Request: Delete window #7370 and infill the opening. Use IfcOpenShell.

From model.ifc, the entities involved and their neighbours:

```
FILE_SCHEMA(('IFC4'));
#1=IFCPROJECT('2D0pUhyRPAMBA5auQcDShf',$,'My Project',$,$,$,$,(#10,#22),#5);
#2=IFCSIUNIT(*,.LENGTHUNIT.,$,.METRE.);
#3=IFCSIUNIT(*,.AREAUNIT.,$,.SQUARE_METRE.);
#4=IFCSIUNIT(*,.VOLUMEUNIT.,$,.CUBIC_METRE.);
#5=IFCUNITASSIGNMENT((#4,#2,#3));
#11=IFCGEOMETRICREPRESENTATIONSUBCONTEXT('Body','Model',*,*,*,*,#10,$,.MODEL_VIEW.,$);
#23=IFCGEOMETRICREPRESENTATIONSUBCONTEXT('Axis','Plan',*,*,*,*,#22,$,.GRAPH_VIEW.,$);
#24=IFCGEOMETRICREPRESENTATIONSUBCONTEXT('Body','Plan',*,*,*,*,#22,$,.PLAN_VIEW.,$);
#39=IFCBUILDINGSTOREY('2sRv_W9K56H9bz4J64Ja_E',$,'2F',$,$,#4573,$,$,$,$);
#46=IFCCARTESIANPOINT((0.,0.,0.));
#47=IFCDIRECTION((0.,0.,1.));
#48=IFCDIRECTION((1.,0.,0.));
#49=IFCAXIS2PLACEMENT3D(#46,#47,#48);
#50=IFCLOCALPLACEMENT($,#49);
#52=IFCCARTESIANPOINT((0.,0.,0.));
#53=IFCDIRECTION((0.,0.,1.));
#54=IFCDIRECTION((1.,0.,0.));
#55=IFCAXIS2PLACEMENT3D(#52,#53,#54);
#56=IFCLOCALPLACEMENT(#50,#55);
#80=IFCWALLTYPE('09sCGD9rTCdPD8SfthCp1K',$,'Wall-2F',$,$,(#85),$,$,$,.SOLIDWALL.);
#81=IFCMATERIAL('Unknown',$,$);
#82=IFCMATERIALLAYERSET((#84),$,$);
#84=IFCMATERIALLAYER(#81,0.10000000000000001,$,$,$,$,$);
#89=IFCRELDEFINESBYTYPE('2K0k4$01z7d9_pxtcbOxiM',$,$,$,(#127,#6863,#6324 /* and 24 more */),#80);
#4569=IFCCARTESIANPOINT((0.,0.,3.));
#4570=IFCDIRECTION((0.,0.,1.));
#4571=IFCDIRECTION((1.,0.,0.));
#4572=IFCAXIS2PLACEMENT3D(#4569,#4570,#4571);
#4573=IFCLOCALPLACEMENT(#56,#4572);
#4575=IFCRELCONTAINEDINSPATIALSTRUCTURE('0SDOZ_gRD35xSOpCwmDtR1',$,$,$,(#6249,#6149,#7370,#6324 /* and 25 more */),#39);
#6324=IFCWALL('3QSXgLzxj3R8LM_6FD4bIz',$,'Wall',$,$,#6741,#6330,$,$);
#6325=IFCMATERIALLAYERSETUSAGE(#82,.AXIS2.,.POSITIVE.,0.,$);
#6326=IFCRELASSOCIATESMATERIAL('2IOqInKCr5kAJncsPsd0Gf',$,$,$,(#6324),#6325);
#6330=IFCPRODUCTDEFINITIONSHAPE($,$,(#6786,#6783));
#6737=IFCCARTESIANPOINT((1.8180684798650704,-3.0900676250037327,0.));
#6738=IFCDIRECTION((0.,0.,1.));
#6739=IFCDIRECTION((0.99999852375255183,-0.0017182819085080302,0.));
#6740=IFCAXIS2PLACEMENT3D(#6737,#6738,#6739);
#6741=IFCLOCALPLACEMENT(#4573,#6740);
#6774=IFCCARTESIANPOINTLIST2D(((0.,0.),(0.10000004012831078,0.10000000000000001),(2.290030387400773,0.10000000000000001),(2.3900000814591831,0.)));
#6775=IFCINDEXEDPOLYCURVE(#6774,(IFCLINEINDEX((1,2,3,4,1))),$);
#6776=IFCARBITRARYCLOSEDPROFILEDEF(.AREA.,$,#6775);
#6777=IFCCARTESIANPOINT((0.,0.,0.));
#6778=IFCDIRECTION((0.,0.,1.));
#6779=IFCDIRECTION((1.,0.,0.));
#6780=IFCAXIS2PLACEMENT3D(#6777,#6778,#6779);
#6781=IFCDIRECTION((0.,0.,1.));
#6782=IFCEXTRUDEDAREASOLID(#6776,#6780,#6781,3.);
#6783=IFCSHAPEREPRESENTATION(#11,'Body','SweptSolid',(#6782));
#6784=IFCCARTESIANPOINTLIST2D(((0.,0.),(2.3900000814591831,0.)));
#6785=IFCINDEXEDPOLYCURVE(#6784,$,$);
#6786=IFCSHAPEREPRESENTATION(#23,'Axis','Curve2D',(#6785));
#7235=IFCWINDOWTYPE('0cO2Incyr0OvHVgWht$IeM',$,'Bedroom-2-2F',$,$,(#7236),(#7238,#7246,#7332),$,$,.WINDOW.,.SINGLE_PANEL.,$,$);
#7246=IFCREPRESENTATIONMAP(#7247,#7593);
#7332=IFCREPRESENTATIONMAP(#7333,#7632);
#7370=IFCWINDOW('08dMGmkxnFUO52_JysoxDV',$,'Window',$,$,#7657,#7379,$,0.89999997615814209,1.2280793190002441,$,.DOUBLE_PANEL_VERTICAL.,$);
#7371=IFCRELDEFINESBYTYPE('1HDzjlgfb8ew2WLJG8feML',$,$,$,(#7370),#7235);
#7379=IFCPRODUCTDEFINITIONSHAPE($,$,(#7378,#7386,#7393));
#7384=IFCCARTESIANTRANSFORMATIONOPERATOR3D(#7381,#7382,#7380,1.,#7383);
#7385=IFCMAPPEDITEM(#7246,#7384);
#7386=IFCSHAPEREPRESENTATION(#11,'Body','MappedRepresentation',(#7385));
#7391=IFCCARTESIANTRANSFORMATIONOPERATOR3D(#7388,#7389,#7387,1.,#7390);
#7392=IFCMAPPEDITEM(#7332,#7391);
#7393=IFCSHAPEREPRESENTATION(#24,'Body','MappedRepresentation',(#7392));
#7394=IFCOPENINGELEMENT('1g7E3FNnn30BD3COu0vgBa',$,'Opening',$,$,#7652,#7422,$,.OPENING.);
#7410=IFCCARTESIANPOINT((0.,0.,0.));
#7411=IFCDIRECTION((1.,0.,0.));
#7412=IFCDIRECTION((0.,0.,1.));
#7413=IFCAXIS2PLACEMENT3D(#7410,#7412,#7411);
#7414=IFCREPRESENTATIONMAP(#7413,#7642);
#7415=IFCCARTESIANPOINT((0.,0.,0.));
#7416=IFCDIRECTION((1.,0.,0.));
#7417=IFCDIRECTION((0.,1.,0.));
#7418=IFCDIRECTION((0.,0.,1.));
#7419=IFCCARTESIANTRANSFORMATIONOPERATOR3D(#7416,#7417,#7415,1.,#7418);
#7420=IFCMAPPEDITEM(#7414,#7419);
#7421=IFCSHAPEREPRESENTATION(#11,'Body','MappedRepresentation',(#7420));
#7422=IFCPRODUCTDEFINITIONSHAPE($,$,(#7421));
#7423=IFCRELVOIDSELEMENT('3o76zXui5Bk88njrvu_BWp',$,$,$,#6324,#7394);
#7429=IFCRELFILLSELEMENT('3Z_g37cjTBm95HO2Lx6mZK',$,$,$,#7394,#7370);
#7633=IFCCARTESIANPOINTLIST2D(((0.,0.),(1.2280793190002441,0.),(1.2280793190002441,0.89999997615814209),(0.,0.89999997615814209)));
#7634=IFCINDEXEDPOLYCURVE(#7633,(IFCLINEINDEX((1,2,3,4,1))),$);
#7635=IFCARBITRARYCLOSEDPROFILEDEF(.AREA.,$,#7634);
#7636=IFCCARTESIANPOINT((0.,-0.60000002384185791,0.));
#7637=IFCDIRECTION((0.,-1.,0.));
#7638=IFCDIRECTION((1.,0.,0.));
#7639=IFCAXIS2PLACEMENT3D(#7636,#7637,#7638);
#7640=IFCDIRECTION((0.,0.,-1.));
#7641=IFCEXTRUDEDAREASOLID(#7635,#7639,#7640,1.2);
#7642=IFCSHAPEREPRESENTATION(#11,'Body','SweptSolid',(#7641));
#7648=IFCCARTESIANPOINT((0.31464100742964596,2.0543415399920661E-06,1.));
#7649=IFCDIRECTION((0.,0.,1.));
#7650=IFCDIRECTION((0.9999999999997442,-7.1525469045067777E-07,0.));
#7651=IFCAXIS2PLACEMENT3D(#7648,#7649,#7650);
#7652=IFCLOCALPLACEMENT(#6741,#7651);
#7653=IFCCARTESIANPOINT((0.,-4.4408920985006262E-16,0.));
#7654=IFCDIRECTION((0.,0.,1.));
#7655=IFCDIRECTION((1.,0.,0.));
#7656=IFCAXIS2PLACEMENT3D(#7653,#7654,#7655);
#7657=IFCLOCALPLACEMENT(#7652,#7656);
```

```python
import ifcopenshell
import ifcopenshell.api.feature
import ifcopenshell.api.root
import ifcopenshell.geom
import ifcopenshell.util.shape

model = ifcopenshell.open("model.ifc")
settings = ifcopenshell.geom.settings()


def volume(element):
    """Net volume in cubic metres, openings subtracted."""
    shape = ifcopenshell.geom.create_shape(settings, element)
    return ifcopenshell.util.shape.get_volume(shape.geometry)


window = model.by_guid("08dMGmkxnFUO52_JysoxDV")
opening = window.FillsVoids[0].RelatingOpeningElement
wall = opening.VoidsElements[0].RelatingBuildingElement
before = volume(wall)

ifcopenshell.api.root.remove_product(model, product=window)
ifcopenshell.api.feature.remove_feature(model, feature=opening)

after = volume(wall)

print(f"wall volume {before:.3f} -> {after:.3f} m3")

model.write("model_edited.ifc")
```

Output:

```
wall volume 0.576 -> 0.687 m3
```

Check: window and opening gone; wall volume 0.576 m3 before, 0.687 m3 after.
